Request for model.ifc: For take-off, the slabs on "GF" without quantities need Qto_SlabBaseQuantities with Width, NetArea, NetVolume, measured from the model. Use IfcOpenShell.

First a look at what the model holds.

```python
import ifcopenshell
import ifcopenshell.util.element
import ifcopenshell.util.unit

model = ifcopenshell.open("model.ifc")
print(model.schema)
for unit_type in ("LENGTHUNIT", "AREAUNIT", "VOLUMEUNIT"):
    print(unit_type, ifcopenshell.util.unit.calculate_unit_scale(model, unit_type))
storey = next(s for s in model.by_type("IfcBuildingStorey") if s.Name == "GF")
slabs = [e for e in ifcopenshell.util.element.get_decomposition(storey) if e.is_a("IfcSlab")]
for e in sorted(slabs, key=lambda e: e.id()):
    print(e.id(), e.is_a(), e.Name, list(ifcopenshell.util.element.get_psets(e, qtos_only=True)), sep=" | ")
```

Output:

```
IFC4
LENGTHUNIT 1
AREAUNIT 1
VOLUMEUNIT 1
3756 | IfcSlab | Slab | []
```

```python
import ifcopenshell
import ifcopenshell.api.pset
import ifcopenshell.geom
import ifcopenshell.util.element
import ifcopenshell.util.shape
import ifcopenshell.util.unit

model = ifcopenshell.open("model.ifc")
unit_scale = ifcopenshell.util.unit.calculate_unit_scale(model)
area_scale = ifcopenshell.util.unit.calculate_unit_scale(model, "AREAUNIT")
volume_scale = ifcopenshell.util.unit.calculate_unit_scale(model, "VOLUMEUNIT")
settings = ifcopenshell.geom.settings()

storey = next(s for s in model.by_type("IfcBuildingStorey") if s.Name == "GF")
slabs = [e for e in ifcopenshell.util.element.get_decomposition(storey) if e.is_a("IfcSlab")]

for e in sorted(slabs, key=lambda e: e.id()):
    if ifcopenshell.util.element.get_psets(e, qtos_only=True, should_inherit=False):
        continue
    # Geometry comes back in metres, in the element's own axes.
    shape = ifcopenshell.geom.create_shape(settings, e)
    values = {
        "Width": ifcopenshell.util.shape.get_z(shape.geometry) / unit_scale,
        "NetArea": ifcopenshell.util.shape.get_footprint_area(shape.geometry) / area_scale,
        "NetVolume": ifcopenshell.util.shape.get_volume(shape.geometry) / volume_scale,
    }
    qto = ifcopenshell.api.pset.add_qto(model, product=e, name="Qto_SlabBaseQuantities")
    ifcopenshell.api.pset.edit_qto(model, qto=qto, properties=values)
    print(e.id(), {k: round(v, 3) for k, v in values.items()})

model.write("model-out.ifc")
```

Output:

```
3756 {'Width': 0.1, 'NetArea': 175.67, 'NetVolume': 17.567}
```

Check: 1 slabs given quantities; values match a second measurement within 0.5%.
